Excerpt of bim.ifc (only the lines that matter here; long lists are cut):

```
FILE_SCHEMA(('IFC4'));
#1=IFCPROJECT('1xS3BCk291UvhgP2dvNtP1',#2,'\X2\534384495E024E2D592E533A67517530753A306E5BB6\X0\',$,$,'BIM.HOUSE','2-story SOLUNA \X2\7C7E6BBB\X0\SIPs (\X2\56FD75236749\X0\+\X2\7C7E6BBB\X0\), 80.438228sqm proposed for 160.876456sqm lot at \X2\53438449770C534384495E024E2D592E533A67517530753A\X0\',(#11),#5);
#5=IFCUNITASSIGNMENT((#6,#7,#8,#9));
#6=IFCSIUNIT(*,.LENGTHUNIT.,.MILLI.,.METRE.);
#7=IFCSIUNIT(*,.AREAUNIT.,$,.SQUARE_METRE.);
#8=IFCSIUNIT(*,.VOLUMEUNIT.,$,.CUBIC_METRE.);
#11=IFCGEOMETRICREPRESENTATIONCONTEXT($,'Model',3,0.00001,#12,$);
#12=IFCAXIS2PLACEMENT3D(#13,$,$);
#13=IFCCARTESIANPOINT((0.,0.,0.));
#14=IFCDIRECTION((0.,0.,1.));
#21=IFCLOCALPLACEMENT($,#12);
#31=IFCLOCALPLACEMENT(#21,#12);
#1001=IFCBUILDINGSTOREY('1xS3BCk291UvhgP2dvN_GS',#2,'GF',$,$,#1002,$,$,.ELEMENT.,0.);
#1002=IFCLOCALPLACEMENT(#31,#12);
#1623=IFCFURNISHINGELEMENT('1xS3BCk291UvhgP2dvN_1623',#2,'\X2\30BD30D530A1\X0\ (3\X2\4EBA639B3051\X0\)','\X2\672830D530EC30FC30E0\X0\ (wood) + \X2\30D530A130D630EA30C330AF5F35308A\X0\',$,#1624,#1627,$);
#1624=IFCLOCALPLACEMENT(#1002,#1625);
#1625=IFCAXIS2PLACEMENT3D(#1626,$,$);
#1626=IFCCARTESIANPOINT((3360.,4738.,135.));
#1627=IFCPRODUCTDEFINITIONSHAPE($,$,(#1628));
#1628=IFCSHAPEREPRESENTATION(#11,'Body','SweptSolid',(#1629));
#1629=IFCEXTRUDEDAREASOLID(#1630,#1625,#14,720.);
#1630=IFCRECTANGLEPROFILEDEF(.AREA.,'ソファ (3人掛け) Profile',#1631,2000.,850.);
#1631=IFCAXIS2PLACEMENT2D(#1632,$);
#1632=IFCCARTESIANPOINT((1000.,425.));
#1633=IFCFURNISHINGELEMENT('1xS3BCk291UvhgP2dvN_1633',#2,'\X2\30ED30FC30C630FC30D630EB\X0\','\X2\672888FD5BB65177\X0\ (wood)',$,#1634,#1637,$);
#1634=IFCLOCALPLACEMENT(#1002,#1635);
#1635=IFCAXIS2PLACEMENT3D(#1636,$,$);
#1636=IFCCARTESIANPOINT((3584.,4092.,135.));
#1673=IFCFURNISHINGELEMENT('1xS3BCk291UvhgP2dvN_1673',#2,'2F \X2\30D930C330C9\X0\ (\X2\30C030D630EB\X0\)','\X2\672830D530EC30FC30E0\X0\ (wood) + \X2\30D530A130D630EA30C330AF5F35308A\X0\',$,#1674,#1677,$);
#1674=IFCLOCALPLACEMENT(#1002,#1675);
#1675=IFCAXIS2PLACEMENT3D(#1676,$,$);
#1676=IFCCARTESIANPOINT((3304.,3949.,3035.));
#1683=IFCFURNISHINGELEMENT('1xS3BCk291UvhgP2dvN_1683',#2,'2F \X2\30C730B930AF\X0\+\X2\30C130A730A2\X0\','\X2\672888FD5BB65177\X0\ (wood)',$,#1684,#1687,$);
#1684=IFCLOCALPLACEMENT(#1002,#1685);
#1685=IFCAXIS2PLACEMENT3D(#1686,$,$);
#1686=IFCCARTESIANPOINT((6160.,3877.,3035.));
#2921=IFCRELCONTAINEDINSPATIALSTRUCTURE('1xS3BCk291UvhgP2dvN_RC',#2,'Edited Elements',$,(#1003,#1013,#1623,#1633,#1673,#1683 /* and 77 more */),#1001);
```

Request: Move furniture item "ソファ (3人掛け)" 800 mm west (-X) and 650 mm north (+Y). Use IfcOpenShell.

```python
import ifcopenshell
import ifcopenshell.api.geometry
import ifcopenshell.util.placement
import ifcopenshell.util.unit

model = ifcopenshell.open("bim.ifc")
unit_scale = ifcopenshell.util.unit.calculate_unit_scale(model)

item = model.by_guid("1xS3BCk291UvhgP2dvN_1623")
matrix = ifcopenshell.util.placement.get_local_placement(item.ObjectPlacement)
matrix[0, 3] -= 0.8 / unit_scale
matrix[1, 3] += 0.65 / unit_scale
ifcopenshell.api.geometry.edit_object_placement(model, product=item, matrix=matrix, is_si=False)

print(ifcopenshell.util.placement.get_local_placement(item.ObjectPlacement).round(3) + 0.0)

model.write("bim_edited.ifc")
```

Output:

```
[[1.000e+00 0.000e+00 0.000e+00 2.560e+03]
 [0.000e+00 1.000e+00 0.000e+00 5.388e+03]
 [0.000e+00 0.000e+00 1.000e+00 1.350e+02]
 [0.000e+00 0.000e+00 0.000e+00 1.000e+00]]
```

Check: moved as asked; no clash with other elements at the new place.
